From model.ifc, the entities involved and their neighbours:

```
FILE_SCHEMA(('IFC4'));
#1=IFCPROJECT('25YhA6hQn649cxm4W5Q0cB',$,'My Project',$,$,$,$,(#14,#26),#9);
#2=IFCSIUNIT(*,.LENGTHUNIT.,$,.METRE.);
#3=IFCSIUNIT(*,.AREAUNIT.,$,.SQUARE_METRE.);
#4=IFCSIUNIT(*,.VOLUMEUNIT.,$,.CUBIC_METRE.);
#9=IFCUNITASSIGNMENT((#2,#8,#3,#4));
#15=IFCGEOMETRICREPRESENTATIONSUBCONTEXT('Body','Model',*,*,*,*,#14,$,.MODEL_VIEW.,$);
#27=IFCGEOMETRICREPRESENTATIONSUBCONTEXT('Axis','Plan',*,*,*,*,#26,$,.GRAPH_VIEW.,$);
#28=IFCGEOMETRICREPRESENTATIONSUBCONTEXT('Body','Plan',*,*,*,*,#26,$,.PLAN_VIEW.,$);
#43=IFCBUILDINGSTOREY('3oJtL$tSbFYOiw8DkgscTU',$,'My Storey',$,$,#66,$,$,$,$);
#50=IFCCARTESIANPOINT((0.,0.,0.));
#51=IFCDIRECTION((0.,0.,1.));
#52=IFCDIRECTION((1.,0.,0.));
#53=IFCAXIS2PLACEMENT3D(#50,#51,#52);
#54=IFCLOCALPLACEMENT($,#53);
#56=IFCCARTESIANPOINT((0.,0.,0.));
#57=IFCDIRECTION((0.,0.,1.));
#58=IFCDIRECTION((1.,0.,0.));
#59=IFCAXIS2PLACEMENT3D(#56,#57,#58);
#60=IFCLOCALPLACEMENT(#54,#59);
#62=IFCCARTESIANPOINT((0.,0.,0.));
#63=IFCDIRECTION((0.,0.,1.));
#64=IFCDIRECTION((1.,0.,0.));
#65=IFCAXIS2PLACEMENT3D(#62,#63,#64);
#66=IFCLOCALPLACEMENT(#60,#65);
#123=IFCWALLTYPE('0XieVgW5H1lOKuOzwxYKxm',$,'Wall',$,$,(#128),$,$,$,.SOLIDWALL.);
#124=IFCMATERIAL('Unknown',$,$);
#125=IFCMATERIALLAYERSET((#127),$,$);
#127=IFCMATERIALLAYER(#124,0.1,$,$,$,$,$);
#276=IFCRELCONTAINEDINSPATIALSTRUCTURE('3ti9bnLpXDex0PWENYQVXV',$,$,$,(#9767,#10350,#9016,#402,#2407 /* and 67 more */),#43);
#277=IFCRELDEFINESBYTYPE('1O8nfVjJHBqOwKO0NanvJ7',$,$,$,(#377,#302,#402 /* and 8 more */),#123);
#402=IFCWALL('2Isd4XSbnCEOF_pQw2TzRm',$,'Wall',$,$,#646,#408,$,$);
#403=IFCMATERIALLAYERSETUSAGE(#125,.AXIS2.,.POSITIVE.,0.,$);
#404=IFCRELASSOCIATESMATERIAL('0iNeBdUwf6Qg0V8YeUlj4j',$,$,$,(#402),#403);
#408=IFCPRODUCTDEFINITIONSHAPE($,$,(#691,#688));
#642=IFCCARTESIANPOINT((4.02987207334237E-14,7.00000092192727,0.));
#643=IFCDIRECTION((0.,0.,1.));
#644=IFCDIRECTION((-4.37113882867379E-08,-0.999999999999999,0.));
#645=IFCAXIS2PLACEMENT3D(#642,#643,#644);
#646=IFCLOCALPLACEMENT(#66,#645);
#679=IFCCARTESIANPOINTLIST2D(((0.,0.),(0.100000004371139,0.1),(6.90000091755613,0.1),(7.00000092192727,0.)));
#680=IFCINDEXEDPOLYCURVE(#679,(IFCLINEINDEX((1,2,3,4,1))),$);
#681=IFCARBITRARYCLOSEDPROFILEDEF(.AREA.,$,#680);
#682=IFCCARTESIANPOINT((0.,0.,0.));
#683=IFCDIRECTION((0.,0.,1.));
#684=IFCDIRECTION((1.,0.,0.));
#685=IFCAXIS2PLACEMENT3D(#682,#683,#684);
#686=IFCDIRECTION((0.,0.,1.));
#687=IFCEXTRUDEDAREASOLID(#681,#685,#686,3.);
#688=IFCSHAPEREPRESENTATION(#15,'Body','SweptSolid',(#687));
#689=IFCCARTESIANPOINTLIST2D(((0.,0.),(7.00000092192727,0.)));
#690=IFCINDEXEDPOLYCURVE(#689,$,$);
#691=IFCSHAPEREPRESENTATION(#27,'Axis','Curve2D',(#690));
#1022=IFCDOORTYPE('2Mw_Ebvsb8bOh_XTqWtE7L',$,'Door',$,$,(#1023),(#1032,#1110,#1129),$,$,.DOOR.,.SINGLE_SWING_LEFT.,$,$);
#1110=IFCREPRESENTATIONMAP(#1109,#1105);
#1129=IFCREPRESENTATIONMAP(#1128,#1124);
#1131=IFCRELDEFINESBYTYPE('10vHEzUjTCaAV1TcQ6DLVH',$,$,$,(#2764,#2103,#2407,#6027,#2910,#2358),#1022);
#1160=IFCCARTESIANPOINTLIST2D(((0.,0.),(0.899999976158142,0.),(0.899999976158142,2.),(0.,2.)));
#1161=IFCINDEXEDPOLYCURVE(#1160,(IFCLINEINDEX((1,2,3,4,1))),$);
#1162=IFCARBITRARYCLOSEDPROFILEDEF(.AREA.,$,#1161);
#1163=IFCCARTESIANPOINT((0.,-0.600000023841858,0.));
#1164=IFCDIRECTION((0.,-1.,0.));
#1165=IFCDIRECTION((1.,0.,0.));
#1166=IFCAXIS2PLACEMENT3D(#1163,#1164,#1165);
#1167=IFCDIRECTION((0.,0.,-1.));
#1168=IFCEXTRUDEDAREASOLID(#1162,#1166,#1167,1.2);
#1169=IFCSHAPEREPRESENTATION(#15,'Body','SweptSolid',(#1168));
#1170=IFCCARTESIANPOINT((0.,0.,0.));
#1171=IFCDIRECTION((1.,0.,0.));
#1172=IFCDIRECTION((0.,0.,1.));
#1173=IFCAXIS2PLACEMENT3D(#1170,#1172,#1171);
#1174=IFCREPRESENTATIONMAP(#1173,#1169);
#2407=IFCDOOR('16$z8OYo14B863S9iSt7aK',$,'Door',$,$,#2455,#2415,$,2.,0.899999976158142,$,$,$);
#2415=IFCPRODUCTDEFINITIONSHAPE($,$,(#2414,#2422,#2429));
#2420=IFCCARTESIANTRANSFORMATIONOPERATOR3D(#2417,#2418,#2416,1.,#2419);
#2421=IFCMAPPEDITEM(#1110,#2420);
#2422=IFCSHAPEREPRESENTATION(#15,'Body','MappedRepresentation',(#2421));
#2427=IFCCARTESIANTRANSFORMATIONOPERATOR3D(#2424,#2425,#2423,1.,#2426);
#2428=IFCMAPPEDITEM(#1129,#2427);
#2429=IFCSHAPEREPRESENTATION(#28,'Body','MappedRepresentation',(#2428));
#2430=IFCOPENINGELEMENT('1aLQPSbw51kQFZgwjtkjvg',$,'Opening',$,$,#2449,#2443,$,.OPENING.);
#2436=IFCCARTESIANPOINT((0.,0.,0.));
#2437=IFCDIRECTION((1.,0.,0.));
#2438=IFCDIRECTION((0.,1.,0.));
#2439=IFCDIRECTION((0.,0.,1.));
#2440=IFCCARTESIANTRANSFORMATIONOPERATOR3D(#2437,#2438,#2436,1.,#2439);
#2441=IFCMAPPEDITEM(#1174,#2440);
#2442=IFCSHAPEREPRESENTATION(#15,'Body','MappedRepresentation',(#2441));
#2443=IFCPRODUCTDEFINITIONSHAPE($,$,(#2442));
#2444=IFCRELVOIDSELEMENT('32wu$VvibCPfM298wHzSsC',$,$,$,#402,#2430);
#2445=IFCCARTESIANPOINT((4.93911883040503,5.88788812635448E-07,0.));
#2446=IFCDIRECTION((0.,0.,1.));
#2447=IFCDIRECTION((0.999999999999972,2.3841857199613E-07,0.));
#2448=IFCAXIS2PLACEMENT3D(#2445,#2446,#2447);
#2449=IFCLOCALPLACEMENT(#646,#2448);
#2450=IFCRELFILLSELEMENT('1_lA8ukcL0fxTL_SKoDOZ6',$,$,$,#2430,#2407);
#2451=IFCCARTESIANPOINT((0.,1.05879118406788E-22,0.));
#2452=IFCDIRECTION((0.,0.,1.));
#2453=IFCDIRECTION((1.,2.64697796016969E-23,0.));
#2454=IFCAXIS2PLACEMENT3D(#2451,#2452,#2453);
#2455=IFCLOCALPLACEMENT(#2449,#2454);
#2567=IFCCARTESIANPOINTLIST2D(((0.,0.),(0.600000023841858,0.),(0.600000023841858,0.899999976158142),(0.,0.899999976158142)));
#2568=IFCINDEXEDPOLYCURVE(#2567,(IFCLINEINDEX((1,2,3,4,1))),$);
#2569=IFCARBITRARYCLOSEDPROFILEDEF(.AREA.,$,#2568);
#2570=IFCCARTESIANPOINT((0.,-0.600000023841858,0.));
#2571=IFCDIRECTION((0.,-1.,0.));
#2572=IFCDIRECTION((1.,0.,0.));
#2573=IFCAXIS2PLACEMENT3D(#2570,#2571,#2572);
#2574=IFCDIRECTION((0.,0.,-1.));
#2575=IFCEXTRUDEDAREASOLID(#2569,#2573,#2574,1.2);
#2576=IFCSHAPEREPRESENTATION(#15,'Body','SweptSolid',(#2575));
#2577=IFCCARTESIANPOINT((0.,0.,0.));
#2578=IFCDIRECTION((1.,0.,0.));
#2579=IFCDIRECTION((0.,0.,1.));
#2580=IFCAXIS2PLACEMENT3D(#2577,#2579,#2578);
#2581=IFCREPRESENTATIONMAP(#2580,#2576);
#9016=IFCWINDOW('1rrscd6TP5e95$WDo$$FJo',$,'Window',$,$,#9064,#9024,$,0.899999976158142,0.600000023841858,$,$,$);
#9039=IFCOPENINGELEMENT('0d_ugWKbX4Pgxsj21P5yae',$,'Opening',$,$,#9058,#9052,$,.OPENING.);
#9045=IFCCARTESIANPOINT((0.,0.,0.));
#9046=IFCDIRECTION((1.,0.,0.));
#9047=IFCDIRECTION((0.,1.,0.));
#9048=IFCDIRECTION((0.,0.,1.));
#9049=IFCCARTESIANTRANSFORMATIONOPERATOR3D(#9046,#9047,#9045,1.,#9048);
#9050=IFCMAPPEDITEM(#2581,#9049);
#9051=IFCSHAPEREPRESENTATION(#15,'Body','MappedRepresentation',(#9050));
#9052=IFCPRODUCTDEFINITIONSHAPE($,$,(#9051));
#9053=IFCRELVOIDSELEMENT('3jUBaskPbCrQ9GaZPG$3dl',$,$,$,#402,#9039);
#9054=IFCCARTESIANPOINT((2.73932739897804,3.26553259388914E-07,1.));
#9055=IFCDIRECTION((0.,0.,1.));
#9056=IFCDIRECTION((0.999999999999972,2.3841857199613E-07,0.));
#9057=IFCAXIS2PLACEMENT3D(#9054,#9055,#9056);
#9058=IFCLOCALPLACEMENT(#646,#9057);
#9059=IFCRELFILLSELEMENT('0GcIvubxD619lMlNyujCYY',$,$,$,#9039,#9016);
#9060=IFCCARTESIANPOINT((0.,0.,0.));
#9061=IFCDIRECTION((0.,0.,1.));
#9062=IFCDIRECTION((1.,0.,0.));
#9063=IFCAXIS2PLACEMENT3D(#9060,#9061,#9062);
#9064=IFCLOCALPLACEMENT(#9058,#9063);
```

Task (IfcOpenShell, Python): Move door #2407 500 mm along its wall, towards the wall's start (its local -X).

```python
import ifcopenshell
import ifcopenshell.api.geometry
import ifcopenshell.util.placement
import ifcopenshell.util.unit

model = ifcopenshell.open("model.ifc")
unit_scale = ifcopenshell.util.unit.calculate_unit_scale(model)

door = model.by_guid("16$z8OYo14B863S9iSt7aK")
opening = door.FillsVoids[0].RelatingOpeningElement
wall = opening.VoidsElements[0].RelatingBuildingElement

wall_matrix = ifcopenshell.util.placement.get_local_placement(wall.ObjectPlacement)
shift = wall_matrix[:3, 0] * -0.5 / unit_scale
before = ifcopenshell.util.placement.get_local_placement(door.ObjectPlacement)[:3, 3].copy()

# The door is placed relative to its opening, so it follows when the opening moves.
matrix = ifcopenshell.util.placement.get_local_placement(opening.ObjectPlacement)
matrix[:3, 3] += shift
ifcopenshell.api.geometry.edit_object_placement(
    model, product=opening, matrix=matrix, is_si=False, should_transform_children=True
)

after = ifcopenshell.util.placement.get_local_placement(door.ObjectPlacement)[:3, 3]
print("door moved by", (after - before).round(3) + 0.0)

model.write("model_updated.ifc")
```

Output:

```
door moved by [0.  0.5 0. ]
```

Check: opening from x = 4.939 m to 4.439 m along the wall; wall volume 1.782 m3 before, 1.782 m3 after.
